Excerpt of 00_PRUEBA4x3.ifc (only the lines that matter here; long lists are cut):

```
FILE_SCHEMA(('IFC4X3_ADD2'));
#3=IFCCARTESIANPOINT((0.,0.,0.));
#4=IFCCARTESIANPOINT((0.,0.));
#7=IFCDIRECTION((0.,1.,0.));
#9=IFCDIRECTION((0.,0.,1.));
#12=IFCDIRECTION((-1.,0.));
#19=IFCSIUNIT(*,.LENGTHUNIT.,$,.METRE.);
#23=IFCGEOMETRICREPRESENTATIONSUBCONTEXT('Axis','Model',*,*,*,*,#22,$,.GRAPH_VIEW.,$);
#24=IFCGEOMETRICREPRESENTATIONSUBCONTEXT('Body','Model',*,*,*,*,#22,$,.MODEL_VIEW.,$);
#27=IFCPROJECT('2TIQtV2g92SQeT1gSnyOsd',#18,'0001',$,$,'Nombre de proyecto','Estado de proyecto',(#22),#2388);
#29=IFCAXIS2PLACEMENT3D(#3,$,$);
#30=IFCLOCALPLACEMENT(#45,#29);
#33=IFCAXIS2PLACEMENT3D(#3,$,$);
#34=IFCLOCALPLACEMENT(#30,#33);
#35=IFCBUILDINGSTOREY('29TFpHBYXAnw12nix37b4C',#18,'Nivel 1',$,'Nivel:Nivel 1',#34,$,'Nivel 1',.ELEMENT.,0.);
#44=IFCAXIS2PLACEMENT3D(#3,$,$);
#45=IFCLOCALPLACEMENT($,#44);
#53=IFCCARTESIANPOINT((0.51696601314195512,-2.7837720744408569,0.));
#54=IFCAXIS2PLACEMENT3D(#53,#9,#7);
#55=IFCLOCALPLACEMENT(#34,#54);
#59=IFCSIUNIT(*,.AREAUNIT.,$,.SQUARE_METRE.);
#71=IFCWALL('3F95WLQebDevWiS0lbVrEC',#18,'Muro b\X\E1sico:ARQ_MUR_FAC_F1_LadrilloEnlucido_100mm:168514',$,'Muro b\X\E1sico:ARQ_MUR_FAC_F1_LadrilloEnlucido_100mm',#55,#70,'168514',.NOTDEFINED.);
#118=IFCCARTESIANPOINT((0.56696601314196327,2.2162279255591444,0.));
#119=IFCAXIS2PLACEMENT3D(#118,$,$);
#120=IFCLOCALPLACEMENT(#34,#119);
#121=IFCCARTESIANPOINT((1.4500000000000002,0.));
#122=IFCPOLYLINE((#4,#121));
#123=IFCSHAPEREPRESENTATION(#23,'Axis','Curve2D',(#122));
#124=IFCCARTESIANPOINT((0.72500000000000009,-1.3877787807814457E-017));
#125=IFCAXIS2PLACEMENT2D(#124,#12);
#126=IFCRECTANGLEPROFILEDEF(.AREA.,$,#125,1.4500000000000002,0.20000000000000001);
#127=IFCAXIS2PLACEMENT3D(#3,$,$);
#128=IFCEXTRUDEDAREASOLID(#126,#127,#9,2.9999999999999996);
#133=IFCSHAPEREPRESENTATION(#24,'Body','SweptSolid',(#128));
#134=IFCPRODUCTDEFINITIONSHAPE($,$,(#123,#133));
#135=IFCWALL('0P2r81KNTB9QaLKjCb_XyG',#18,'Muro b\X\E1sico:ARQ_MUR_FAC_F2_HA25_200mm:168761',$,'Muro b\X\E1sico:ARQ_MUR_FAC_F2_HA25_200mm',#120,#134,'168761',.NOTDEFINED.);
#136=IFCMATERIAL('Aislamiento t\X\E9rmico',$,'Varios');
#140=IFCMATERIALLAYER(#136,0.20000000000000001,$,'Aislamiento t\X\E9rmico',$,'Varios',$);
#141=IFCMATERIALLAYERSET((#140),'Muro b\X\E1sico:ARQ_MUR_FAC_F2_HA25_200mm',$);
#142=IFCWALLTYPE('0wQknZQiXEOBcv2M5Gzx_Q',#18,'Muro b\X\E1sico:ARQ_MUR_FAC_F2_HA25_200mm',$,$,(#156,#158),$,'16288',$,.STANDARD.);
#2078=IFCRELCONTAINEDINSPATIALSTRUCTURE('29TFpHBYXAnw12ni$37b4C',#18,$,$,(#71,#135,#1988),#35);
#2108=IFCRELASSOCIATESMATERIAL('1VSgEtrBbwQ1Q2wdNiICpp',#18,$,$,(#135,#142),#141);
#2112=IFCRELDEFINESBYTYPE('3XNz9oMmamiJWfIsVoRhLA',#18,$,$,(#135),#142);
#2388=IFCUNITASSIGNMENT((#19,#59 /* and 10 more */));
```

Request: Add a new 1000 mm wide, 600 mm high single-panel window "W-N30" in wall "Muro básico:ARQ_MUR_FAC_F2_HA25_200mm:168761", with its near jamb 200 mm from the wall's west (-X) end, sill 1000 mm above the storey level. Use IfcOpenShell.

```python
import numpy as np
import ifcopenshell
import ifcopenshell.api.feature
import ifcopenshell.api.geometry
import ifcopenshell.api.root
import ifcopenshell.api.spatial
import ifcopenshell.geom
import ifcopenshell.util.element
import ifcopenshell.util.placement
import ifcopenshell.util.representation
import ifcopenshell.util.shape
import ifcopenshell.util.unit

model = ifcopenshell.open("00_PRUEBA4x3.ifc")
unit_scale = ifcopenshell.util.unit.calculate_unit_scale(model)
settings = ifcopenshell.geom.settings()


def volume(element):
    """Net volume in cubic metres, openings subtracted."""
    shape = ifcopenshell.geom.create_shape(settings, element)
    return ifcopenshell.util.shape.get_volume(shape.geometry)


wall = model.by_guid("0P2r81KNTB9QaLKjCb_XyG")
storey = ifcopenshell.util.element.get_container(wall, ifc_class="IfcBuildingStorey")
context = ifcopenshell.util.representation.get_context(model, "Model", "Body", "MODEL_VIEW")
before = volume(wall)

width, height, from_end, sill = 1, 0.6, 0.2, 1  # metres

# The wall runs along its own X axis, and the end named is its -X end.
wall_shape = ifcopenshell.geom.create_shape(settings, wall)
x, y, z = ifcopenshell.util.shape.get_vertices(wall_shape.geometry).T
start = x.min() + from_end
face, thickness = float(y.min()), float(y.max() - y.min())
wall_matrix = ifcopenshell.util.placement.get_local_placement(wall.ObjectPlacement)
level = ifcopenshell.util.placement.get_local_placement(storey.ObjectPlacement)[2, 3]


def in_wall(x, y):
    """Placement at x, y metres in the wall's axes, at sill height."""
    matrix = wall_matrix.copy()
    matrix[:, 3] = wall_matrix @ np.array([x / unit_scale, y / unit_scale, 0.0, 1.0])
    matrix[2, 3] = level + sill / unit_scale
    return matrix


# Opening: a box that overshoots both wall faces by 50 mm.
opening = ifcopenshell.api.root.create_entity(model, ifc_class="IfcOpeningElement", predefined_type="OPENING")
box = ifcopenshell.api.geometry.add_wall_representation(
    model, context=context, length=width, height=height, thickness=thickness + 0.1
)
ifcopenshell.api.geometry.assign_representation(model, product=opening, representation=box)
ifcopenshell.api.geometry.edit_object_placement(model, product=opening, matrix=in_wall(start, face - 0.05), is_si=False)
ifcopenshell.api.feature.add_feature(model, feature=opening, element=wall)

window = ifcopenshell.api.root.create_entity(model, ifc_class="IfcWindow", name="W-N30", predefined_type="WINDOW")
window.OverallWidth, window.OverallHeight = width / unit_scale, height / unit_scale
window.PartitioningType = "SINGLE_PANEL"
body = ifcopenshell.api.geometry.add_window_representation(
    model,
    context=context,
    overall_width=window.OverallWidth,
    overall_height=window.OverallHeight,
    partition_type="SINGLE_PANEL",
)
ifcopenshell.api.geometry.assign_representation(model, product=window, representation=body)
ifcopenshell.api.spatial.assign_container(model, products=[window], relating_structure=storey)
ifcopenshell.api.feature.add_filling(model, opening=opening, element=window)

# Centre the window in the wall's thickness.
ifcopenshell.api.geometry.edit_object_placement(model, product=window, matrix=in_wall(start, face), is_si=False)
window_shape = ifcopenshell.geom.create_shape(settings, window)
depth = ifcopenshell.util.shape.get_vertices(window_shape.geometry)[:, 1]
offset = face + thickness / 2 - (depth.min() + depth.max()) / 2
ifcopenshell.api.geometry.edit_object_placement(model, product=window, matrix=in_wall(start, offset), is_si=False)

after = volume(wall)

print(f"wall volume {before:.3f} -> {after:.3f} m3")

model.write("00_PRUEBA4x3_edited.ifc")
```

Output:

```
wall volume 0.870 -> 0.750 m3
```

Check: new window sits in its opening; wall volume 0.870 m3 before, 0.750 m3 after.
